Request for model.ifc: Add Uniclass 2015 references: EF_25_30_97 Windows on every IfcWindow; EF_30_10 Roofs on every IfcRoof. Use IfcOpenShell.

First a look at what the model holds.

```python
import ifcopenshell

model = ifcopenshell.open("model.ifc")
print(model.schema)
print("classifications:", [c.Name for c in model.by_type("IfcClassification")])
for ifc_class in ("IfcDoor", "IfcRoof", "IfcStair", "IfcWall", "IfcWindow"):
    print(ifc_class, len(model.by_type(ifc_class)))
```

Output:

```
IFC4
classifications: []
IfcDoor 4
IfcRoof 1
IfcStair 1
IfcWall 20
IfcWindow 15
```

```python
import ifcopenshell
import ifcopenshell.api.classification

model = ifcopenshell.open("model.ifc")

system = ifcopenshell.api.classification.add_classification(model, classification="Uniclass 2015")

codes = {
    "IfcWindow": ("EF_25_30_97", "Windows"),
    "IfcRoof": ("EF_30_10", "Roofs"),
}
for ifc_class, (code, name) in codes.items():
    products = model.by_type(ifc_class)
    ifcopenshell.api.classification.add_reference(
        model, products=products, classification=system, identification=code, name=name
    )
    print(code, len(products))

model.write("model_rev.ifc")
```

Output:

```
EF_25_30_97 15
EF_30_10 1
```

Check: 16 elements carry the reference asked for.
